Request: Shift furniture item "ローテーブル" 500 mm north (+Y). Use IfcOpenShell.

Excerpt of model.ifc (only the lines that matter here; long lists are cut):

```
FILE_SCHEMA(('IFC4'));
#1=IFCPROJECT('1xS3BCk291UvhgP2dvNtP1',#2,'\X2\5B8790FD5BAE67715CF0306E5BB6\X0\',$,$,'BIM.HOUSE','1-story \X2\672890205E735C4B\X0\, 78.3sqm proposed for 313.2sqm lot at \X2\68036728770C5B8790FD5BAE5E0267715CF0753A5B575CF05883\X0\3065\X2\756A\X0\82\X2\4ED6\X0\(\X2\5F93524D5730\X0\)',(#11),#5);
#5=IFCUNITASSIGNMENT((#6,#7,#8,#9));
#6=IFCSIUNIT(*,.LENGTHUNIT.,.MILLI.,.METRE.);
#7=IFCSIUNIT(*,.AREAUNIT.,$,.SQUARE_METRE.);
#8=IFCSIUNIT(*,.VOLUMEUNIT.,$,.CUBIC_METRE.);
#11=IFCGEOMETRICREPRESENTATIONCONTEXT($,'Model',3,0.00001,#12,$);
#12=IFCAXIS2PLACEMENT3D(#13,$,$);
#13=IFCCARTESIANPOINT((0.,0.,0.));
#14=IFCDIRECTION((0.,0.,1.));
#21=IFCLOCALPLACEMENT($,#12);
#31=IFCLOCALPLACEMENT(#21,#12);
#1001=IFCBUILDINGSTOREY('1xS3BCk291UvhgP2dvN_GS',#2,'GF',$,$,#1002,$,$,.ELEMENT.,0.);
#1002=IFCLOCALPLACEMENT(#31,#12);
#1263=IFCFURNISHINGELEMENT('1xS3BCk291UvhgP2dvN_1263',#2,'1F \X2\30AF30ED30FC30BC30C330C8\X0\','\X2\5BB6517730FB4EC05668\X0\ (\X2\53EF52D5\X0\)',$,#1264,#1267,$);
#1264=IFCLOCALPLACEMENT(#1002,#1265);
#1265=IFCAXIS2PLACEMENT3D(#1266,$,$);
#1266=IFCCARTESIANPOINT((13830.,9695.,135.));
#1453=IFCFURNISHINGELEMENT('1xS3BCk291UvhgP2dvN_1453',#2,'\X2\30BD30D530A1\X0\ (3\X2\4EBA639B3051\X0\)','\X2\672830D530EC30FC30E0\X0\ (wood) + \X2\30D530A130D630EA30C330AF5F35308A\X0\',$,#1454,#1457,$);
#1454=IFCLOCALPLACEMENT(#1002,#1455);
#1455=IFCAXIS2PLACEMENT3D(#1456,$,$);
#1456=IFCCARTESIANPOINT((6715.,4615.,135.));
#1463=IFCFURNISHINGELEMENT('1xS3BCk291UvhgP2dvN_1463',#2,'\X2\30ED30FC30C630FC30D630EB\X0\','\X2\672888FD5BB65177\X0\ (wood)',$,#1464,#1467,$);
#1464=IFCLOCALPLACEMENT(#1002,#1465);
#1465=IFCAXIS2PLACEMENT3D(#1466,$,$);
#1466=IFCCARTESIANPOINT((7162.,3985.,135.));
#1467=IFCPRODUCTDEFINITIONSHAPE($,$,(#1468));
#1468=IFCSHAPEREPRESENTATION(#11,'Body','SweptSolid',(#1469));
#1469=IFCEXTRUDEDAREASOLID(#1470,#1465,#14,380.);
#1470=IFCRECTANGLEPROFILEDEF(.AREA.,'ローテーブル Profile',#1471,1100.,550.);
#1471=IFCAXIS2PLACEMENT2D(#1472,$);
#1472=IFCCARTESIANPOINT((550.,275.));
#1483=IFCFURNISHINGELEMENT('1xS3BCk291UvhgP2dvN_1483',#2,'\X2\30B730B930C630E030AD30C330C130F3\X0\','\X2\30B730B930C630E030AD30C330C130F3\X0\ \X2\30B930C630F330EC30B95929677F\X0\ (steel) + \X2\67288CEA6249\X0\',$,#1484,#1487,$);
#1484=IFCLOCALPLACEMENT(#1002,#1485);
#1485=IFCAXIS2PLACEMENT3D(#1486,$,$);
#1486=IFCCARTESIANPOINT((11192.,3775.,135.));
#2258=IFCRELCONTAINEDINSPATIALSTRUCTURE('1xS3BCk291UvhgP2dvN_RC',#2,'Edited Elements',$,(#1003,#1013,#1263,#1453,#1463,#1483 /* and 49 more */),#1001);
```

```python
import ifcopenshell
import ifcopenshell.api.geometry
import ifcopenshell.util.placement
import ifcopenshell.util.unit

model = ifcopenshell.open("model.ifc")
unit_scale = ifcopenshell.util.unit.calculate_unit_scale(model)

item = model.by_guid("1xS3BCk291UvhgP2dvN_1463")
matrix = ifcopenshell.util.placement.get_local_placement(item.ObjectPlacement)
matrix[1, 3] += 0.5 / unit_scale
ifcopenshell.api.geometry.edit_object_placement(model, product=item, matrix=matrix, is_si=False)

print(ifcopenshell.util.placement.get_local_placement(item.ObjectPlacement).round(3) + 0.0)

model.write("model_updated.ifc")
```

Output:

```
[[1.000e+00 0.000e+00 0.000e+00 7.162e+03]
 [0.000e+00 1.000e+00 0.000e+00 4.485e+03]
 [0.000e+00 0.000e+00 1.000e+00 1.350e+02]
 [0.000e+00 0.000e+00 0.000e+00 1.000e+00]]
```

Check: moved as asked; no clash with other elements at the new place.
